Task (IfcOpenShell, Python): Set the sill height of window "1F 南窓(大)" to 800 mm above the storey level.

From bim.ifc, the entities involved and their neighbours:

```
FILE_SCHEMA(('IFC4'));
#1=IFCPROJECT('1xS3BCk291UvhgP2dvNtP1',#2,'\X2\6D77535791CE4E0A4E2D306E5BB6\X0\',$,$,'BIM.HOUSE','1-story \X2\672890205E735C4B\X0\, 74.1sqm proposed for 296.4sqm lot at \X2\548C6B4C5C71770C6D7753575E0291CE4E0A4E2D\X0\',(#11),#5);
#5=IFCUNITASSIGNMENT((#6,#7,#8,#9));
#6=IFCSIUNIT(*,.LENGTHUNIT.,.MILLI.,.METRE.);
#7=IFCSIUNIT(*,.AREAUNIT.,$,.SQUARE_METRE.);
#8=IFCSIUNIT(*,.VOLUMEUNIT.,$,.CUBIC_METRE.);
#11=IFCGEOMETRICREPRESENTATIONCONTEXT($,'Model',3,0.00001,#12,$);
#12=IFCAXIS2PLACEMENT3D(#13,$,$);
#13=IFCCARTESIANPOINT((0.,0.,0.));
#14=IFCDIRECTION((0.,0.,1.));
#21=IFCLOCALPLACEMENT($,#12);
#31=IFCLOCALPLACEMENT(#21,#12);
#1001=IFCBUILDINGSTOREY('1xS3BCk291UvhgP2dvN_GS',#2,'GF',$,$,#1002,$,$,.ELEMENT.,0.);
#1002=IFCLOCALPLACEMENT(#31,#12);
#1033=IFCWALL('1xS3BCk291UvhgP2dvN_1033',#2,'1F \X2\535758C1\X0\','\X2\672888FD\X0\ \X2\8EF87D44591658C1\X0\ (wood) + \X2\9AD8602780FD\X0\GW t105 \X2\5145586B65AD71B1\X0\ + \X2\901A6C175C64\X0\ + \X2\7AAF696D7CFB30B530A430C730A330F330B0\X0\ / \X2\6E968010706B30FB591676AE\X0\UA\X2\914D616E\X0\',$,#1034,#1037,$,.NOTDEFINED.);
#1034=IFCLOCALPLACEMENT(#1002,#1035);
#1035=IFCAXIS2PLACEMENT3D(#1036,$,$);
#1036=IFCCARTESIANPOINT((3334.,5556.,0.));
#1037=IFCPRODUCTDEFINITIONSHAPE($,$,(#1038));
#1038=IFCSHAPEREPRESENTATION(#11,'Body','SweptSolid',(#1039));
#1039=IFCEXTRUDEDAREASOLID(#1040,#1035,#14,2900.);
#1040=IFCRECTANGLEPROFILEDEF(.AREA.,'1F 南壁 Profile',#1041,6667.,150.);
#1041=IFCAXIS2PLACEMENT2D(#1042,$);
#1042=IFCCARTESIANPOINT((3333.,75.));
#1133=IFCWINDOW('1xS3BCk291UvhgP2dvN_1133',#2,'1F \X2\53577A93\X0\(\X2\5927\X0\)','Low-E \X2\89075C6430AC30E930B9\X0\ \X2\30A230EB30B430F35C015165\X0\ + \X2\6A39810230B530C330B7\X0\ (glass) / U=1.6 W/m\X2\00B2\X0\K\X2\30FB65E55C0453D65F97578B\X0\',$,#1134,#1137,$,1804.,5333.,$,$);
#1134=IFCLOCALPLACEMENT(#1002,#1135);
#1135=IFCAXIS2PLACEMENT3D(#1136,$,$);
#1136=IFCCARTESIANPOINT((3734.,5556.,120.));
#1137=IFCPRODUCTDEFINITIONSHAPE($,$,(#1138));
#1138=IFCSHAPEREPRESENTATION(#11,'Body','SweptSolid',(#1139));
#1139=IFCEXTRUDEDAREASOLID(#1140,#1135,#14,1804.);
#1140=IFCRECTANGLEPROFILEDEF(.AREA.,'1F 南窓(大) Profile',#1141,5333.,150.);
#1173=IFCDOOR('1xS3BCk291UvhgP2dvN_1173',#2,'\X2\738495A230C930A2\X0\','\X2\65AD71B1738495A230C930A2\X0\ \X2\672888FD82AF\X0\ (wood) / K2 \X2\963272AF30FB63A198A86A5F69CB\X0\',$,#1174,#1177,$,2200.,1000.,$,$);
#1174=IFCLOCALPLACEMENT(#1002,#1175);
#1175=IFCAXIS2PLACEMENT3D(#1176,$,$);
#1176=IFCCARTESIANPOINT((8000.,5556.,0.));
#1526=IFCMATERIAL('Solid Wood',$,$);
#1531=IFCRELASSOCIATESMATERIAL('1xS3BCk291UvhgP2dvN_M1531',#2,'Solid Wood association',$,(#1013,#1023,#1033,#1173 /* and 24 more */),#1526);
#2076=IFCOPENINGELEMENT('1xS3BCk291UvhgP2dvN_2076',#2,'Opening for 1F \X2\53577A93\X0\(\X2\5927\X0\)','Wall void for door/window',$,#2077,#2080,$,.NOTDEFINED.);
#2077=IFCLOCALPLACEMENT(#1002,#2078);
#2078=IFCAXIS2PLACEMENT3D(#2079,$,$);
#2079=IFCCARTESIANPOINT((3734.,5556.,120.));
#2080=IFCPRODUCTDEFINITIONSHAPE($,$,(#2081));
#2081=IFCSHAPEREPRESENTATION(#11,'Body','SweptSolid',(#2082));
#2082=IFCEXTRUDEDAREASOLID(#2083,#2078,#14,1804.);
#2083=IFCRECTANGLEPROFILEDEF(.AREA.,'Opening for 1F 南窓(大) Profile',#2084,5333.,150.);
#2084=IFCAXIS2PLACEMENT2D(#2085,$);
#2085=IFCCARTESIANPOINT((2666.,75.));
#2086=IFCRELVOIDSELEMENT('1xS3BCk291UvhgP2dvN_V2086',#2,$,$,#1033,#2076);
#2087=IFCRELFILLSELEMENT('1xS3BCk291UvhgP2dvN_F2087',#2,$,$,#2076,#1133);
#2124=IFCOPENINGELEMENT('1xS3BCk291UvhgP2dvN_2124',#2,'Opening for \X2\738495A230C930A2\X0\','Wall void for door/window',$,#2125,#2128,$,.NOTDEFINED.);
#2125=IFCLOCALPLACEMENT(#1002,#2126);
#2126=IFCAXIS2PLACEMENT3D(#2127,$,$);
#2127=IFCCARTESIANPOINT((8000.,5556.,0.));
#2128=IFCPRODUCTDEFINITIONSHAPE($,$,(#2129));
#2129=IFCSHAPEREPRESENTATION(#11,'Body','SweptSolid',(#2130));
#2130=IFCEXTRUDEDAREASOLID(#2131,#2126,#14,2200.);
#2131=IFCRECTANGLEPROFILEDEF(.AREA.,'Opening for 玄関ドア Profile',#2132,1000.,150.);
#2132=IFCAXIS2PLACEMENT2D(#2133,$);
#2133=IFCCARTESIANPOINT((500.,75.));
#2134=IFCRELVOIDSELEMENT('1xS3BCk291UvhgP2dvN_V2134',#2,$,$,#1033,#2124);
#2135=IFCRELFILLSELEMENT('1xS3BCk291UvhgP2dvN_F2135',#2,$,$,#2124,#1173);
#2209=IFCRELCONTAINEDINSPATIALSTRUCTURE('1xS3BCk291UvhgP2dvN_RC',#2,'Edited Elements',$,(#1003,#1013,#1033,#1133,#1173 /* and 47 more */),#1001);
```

```python
import numpy as np
import ifcopenshell
import ifcopenshell.api.geometry
import ifcopenshell.geom
import ifcopenshell.util.element
import ifcopenshell.util.placement
import ifcopenshell.util.shape
import ifcopenshell.util.unit

model = ifcopenshell.open("bim.ifc")
unit_scale = ifcopenshell.util.unit.calculate_unit_scale(model)

window = model.by_guid("1xS3BCk291UvhgP2dvN_1133")
opening = window.FillsVoids[0].RelatingOpeningElement
storey = ifcopenshell.util.element.get_container(window, ifc_class="IfcBuildingStorey")
level = ifcopenshell.util.placement.get_local_placement(storey.ObjectPlacement)[2, 3]

# The opening's origin need not be at the sill, so measure its lowest point.
shape = ifcopenshell.geom.create_shape(ifcopenshell.geom.settings(), opening)
bottom = ifcopenshell.util.shape.get_shape_bottom_elevation(shape, shape.geometry) / unit_scale
dz = level + 0.8 / unit_scale - bottom

shift = np.array([0.0, 0.0, dz])
# The window is not placed relative to its opening, so move both.
for product in (opening, window):
    matrix = ifcopenshell.util.placement.get_local_placement(product.ObjectPlacement)
    matrix[:3, 3] += shift
    ifcopenshell.api.geometry.edit_object_placement(model, product=product, matrix=matrix, is_si=False)

print(f"moved by {dz * unit_scale:+.3f} m")

model.write("bim_edited.ifc")
```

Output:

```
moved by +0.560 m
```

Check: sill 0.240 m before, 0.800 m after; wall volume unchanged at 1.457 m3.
